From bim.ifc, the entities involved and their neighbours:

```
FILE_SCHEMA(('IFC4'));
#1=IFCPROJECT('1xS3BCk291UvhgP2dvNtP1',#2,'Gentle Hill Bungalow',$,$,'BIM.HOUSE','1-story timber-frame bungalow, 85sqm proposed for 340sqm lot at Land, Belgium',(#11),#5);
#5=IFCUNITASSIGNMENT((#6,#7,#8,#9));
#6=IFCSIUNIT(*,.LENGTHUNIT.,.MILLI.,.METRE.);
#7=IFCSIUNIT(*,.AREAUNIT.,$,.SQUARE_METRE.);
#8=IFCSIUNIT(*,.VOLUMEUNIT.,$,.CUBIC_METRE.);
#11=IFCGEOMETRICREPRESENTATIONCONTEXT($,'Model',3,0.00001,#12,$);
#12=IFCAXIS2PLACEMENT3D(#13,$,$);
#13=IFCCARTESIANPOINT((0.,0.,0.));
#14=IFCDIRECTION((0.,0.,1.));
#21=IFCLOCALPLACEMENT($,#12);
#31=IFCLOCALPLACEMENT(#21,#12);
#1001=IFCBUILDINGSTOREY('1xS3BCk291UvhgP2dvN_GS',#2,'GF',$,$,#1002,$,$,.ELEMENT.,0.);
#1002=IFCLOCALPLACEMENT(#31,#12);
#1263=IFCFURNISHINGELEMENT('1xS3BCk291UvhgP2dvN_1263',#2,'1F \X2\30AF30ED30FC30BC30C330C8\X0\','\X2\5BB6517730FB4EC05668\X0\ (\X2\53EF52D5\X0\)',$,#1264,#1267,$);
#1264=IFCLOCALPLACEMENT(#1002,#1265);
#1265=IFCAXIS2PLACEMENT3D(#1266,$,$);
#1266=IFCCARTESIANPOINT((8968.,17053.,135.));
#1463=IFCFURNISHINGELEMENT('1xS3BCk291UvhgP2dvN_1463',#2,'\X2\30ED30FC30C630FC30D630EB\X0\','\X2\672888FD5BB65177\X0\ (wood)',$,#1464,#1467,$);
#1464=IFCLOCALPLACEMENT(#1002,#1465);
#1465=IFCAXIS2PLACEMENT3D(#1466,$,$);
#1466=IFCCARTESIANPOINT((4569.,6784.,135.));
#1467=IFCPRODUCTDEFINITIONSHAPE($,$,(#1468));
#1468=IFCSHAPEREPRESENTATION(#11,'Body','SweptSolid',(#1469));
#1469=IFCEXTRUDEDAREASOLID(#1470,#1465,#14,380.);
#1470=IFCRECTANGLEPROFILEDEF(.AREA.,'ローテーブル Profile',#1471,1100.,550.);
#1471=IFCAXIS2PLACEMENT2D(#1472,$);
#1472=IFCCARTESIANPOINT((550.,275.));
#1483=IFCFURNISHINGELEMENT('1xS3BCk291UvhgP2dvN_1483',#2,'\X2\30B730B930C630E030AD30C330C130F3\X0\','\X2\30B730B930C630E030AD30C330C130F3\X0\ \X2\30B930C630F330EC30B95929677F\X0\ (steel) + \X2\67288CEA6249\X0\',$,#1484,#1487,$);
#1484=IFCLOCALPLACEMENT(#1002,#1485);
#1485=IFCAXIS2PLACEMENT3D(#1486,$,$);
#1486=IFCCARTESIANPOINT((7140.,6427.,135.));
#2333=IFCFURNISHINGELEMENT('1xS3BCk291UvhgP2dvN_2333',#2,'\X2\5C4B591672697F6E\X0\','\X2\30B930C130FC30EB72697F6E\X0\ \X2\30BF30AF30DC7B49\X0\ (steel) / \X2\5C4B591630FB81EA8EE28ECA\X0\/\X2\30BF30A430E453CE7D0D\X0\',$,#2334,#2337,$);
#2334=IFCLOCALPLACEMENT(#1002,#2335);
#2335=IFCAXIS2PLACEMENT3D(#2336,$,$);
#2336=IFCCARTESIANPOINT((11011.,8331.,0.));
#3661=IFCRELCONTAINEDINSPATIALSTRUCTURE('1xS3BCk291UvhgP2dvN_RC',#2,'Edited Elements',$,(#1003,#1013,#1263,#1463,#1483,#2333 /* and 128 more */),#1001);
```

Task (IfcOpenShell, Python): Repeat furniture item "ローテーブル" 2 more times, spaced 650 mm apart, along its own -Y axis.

```python
import ifcopenshell
import ifcopenshell.api.geometry
import ifcopenshell.api.root
import ifcopenshell.util.element
import ifcopenshell.util.placement
import ifcopenshell.util.unit

model = ifcopenshell.open("bim.ifc")
unit_scale = ifcopenshell.util.unit.calculate_unit_scale(model)


def reuse_history(source, copy):
    """copy_class also copies each property set's owner history, people and application; keep the originals."""
    for rel in copy.IsDefinedBy:
        if rel.is_a("IfcRelDefinesByProperties") and (history := rel.RelatingPropertyDefinition.OwnerHistory):
            rel.RelatingPropertyDefinition.OwnerHistory = source.OwnerHistory
            ifcopenshell.util.element.remove_deep2(model, history)


source = model.by_guid("1xS3BCk291UvhgP2dvN_1463")
base = ifcopenshell.util.placement.get_local_placement(source.ObjectPlacement)
step = -base[:3, 1] * 0.65 / unit_scale

for i in range(1, 3):
    copy = ifcopenshell.api.root.copy_class(model, product=source)
    copy.Representation = ifcopenshell.util.element.copy_deep(
        model, source.Representation, exclude=["IfcGeometricRepresentationContext", "IfcRepresentationMap"]
    )
    reuse_history(source, copy)
    matrix = base.copy()
    matrix[:3, 3] += i * step
    print("added at", matrix[:3, 3].round(3) + 0.0)
    ifcopenshell.api.geometry.edit_object_placement(model, product=copy, matrix=matrix, is_si=False)

model.write("bim_rev.ifc")
```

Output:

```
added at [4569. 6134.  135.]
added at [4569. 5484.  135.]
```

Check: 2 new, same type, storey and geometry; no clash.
